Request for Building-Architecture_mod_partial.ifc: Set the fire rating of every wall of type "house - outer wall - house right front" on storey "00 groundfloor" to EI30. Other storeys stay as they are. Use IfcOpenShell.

First a look at what the model holds.

```python
import ifcopenshell
import ifcopenshell.util.element

model = ifcopenshell.open("Building-Architecture_mod_partial.ifc")
print(model.schema)
storey = next(s for s in model.by_type("IfcBuildingStorey") if s.Name == "00 groundfloor")
walls = [e for e in ifcopenshell.util.element.get_decomposition(storey) if e.is_a("IfcWall")]
seen = {}
for e in walls:
    element_type = ifcopenshell.util.element.get_type(e)
    key = (element_type.Name if element_type != e and element_type else None, ifcopenshell.util.element.get_pset(e, "Pset_WallCommon", "FireRating"))
    seen[key] = seen.get(key, 0) + 1
for (name, value), count in sorted(seen.items(), key=str):
    print(count, "x", name, "|", value)
```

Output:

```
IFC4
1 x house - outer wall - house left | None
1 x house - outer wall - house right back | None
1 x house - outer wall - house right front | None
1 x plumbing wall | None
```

```python
import ifcopenshell
import ifcopenshell.api.pset
import ifcopenshell.util.element

model = ifcopenshell.open("Building-Architecture_mod_partial.ifc")

storey = next(s for s in model.by_type("IfcBuildingStorey") if s.Name == "00 groundfloor")
walls = [e for e in ifcopenshell.util.element.get_decomposition(storey) if e.is_a("IfcWall")]

count = 0
for e in walls:
    element_type = ifcopenshell.util.element.get_type(e)
    if element_type in (None, e) or element_type.Name != "house - outer wall - house right front":
        continue
    # add_pset returns the element's existing set when there is one.
    pset = ifcopenshell.api.pset.add_pset(model, product=e, name="Pset_WallCommon")
    ifcopenshell.api.pset.edit_pset(model, pset=pset, properties={"FireRating": "EI30"})
    count += 1

print(count, "walls updated")

model.write("Building-Architecture_mod_partial-out.ifc")
```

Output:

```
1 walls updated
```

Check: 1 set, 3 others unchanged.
